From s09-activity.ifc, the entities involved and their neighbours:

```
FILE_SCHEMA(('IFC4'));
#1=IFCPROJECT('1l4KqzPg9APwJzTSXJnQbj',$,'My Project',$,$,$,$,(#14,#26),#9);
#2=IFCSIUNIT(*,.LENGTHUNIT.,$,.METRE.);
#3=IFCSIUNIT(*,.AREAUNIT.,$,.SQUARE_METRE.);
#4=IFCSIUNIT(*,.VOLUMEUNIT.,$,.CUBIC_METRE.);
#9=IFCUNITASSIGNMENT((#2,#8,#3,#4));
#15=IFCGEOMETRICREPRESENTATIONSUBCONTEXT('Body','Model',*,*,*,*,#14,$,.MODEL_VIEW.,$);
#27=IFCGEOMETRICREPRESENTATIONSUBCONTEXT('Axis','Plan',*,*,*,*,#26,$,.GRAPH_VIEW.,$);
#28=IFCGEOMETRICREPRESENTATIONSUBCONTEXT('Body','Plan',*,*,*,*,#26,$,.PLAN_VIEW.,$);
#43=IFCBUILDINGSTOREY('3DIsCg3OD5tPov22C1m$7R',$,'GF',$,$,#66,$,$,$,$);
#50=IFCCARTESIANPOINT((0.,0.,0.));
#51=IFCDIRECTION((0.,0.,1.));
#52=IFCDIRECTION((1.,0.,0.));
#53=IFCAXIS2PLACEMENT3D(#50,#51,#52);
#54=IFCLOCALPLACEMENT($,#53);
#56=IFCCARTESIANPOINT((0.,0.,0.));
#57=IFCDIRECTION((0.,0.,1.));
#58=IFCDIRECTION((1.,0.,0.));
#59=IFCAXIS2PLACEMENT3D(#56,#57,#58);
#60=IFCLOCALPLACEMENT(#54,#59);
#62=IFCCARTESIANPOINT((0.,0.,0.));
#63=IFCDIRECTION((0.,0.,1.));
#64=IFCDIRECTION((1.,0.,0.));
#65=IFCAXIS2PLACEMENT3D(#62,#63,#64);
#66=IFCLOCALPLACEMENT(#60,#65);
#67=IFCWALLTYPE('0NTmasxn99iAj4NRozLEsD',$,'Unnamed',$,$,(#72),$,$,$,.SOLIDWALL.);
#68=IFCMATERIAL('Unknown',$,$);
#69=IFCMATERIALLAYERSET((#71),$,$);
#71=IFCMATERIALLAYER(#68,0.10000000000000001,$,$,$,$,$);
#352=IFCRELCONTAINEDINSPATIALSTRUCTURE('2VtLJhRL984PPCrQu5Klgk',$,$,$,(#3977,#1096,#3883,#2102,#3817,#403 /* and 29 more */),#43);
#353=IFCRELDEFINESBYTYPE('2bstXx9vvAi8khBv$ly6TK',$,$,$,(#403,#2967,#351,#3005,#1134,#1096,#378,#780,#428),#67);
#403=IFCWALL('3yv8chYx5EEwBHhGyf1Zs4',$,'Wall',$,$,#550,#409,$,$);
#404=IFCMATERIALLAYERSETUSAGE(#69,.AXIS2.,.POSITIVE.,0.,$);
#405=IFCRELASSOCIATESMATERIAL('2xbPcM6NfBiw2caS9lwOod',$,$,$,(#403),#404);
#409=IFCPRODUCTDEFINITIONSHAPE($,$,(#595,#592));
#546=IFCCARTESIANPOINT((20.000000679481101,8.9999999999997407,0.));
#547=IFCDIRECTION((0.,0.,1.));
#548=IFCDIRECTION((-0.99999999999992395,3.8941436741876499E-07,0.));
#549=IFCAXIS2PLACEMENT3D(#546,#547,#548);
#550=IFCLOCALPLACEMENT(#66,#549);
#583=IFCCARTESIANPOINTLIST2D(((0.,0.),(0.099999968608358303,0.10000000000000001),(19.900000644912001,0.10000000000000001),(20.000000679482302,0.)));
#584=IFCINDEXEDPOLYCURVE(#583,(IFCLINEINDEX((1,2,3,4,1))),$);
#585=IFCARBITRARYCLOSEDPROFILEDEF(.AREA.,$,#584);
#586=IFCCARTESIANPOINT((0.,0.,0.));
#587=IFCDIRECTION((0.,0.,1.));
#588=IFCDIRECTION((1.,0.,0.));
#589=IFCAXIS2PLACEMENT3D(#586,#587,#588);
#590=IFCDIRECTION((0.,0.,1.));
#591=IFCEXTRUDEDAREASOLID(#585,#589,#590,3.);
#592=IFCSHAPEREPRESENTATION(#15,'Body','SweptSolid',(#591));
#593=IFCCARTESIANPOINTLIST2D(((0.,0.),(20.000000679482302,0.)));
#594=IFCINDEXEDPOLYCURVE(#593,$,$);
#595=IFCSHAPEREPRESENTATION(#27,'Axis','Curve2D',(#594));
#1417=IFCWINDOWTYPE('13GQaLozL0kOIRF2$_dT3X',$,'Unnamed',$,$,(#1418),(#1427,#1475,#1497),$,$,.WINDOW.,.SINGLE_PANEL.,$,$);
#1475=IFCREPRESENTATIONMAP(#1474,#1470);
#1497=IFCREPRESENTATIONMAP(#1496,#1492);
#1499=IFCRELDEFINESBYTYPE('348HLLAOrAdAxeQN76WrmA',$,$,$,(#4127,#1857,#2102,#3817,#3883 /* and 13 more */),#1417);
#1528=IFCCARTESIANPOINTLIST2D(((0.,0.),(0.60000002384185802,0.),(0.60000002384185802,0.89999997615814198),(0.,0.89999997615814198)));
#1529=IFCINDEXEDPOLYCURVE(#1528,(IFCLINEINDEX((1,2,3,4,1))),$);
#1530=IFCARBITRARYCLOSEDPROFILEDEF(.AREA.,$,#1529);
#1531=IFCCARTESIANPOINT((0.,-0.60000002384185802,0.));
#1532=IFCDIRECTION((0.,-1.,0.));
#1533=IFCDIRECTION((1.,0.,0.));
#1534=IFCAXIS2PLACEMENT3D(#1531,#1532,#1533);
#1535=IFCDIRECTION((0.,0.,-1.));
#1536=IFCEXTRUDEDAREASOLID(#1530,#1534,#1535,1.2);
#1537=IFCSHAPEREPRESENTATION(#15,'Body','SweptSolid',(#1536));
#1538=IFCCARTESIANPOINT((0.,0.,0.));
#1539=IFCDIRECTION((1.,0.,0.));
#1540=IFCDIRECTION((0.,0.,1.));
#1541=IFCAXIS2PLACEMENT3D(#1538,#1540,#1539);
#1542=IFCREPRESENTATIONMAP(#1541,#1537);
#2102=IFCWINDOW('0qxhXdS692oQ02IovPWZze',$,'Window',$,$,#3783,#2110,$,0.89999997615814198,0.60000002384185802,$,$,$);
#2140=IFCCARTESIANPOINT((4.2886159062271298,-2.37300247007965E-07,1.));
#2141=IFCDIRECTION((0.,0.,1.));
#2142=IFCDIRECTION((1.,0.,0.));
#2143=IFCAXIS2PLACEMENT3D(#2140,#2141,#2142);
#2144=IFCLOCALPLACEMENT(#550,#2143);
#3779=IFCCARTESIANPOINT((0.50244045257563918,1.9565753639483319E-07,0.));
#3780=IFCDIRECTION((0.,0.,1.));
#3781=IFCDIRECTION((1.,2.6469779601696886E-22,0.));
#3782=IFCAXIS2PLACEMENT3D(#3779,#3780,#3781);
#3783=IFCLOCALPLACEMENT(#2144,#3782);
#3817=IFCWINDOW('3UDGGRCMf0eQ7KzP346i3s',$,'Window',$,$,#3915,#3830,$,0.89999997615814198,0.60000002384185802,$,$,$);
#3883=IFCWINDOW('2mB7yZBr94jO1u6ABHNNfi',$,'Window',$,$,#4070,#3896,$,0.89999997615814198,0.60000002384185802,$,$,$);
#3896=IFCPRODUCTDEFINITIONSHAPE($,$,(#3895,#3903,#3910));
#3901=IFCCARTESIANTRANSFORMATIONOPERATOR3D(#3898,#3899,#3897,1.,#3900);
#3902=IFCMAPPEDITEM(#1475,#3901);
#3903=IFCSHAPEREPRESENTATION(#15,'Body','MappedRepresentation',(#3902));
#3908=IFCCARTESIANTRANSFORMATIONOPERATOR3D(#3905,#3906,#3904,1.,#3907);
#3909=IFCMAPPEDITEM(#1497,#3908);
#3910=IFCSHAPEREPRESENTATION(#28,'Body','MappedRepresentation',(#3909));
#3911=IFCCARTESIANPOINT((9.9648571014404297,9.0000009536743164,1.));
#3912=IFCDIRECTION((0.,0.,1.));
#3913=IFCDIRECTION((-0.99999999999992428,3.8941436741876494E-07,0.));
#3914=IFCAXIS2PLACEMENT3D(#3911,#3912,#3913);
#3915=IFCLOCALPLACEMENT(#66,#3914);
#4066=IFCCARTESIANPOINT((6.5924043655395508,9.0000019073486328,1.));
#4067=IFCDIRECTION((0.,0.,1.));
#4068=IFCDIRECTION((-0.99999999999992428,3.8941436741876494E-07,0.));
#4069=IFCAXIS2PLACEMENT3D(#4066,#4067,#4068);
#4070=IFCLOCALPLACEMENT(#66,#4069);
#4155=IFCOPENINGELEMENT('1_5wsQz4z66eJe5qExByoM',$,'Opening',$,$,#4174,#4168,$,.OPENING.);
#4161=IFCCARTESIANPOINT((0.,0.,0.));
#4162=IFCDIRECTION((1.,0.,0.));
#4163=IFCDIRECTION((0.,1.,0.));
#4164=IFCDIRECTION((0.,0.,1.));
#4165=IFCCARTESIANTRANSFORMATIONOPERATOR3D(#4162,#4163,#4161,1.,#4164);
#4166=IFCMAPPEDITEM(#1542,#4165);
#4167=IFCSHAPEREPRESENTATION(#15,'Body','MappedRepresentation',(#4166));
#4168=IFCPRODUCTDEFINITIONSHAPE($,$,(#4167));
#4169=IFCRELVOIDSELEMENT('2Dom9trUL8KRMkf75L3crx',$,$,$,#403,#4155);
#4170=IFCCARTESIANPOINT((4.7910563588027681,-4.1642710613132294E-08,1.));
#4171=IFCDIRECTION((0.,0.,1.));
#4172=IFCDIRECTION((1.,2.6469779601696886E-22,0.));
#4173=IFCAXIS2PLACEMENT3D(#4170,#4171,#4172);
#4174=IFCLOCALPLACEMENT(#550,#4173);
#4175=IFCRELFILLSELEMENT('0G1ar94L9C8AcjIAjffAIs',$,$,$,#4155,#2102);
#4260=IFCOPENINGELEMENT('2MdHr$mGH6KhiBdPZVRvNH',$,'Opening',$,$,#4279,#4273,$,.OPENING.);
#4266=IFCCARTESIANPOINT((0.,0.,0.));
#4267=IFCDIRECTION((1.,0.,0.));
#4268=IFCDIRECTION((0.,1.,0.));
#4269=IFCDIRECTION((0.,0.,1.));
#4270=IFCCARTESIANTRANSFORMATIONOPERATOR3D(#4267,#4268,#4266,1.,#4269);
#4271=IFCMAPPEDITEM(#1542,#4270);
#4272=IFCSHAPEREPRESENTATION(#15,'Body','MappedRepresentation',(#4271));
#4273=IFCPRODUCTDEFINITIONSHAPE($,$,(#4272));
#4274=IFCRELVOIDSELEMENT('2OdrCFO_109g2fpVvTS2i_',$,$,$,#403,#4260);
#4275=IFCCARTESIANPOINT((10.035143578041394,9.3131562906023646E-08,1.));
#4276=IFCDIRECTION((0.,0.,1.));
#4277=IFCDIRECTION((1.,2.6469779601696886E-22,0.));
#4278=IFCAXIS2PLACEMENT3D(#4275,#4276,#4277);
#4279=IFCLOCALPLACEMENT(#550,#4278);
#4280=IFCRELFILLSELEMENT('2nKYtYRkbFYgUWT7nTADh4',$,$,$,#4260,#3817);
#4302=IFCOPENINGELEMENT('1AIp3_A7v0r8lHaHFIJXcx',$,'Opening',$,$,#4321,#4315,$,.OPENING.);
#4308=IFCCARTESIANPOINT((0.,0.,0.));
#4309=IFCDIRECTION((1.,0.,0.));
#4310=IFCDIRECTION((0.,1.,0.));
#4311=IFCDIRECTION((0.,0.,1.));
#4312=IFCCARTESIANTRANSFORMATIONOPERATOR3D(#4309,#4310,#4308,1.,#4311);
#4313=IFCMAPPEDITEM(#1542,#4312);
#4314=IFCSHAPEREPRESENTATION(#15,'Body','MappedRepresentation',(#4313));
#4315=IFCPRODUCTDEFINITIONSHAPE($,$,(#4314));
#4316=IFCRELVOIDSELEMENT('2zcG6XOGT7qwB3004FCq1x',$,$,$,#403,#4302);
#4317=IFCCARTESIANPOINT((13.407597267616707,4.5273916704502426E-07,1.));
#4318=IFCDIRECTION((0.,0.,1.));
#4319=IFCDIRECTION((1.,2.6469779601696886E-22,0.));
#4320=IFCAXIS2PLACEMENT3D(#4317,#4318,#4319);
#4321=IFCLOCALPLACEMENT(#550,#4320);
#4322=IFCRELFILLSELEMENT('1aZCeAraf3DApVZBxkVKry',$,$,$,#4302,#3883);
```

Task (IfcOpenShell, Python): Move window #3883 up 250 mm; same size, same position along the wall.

```python
import numpy as np
import ifcopenshell
import ifcopenshell.api.geometry
import ifcopenshell.util.placement
import ifcopenshell.util.unit

model = ifcopenshell.open("s09-activity.ifc")
unit_scale = ifcopenshell.util.unit.calculate_unit_scale(model)

window = model.by_guid("2mB7yZBr94jO1u6ABHNNfi")
opening = window.FillsVoids[0].RelatingOpeningElement
dz = 0.25 / unit_scale

shift = np.array([0.0, 0.0, dz])
# The window is not placed relative to its opening, so move both.
for product in (opening, window):
    matrix = ifcopenshell.util.placement.get_local_placement(product.ObjectPlacement)
    matrix[:3, 3] += shift
    ifcopenshell.api.geometry.edit_object_placement(model, product=product, matrix=matrix, is_si=False)

print(f"moved by {dz * unit_scale:+.3f} m")

model.write("s09-activity_updated.ifc")
```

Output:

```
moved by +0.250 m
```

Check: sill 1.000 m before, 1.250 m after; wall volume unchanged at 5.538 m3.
